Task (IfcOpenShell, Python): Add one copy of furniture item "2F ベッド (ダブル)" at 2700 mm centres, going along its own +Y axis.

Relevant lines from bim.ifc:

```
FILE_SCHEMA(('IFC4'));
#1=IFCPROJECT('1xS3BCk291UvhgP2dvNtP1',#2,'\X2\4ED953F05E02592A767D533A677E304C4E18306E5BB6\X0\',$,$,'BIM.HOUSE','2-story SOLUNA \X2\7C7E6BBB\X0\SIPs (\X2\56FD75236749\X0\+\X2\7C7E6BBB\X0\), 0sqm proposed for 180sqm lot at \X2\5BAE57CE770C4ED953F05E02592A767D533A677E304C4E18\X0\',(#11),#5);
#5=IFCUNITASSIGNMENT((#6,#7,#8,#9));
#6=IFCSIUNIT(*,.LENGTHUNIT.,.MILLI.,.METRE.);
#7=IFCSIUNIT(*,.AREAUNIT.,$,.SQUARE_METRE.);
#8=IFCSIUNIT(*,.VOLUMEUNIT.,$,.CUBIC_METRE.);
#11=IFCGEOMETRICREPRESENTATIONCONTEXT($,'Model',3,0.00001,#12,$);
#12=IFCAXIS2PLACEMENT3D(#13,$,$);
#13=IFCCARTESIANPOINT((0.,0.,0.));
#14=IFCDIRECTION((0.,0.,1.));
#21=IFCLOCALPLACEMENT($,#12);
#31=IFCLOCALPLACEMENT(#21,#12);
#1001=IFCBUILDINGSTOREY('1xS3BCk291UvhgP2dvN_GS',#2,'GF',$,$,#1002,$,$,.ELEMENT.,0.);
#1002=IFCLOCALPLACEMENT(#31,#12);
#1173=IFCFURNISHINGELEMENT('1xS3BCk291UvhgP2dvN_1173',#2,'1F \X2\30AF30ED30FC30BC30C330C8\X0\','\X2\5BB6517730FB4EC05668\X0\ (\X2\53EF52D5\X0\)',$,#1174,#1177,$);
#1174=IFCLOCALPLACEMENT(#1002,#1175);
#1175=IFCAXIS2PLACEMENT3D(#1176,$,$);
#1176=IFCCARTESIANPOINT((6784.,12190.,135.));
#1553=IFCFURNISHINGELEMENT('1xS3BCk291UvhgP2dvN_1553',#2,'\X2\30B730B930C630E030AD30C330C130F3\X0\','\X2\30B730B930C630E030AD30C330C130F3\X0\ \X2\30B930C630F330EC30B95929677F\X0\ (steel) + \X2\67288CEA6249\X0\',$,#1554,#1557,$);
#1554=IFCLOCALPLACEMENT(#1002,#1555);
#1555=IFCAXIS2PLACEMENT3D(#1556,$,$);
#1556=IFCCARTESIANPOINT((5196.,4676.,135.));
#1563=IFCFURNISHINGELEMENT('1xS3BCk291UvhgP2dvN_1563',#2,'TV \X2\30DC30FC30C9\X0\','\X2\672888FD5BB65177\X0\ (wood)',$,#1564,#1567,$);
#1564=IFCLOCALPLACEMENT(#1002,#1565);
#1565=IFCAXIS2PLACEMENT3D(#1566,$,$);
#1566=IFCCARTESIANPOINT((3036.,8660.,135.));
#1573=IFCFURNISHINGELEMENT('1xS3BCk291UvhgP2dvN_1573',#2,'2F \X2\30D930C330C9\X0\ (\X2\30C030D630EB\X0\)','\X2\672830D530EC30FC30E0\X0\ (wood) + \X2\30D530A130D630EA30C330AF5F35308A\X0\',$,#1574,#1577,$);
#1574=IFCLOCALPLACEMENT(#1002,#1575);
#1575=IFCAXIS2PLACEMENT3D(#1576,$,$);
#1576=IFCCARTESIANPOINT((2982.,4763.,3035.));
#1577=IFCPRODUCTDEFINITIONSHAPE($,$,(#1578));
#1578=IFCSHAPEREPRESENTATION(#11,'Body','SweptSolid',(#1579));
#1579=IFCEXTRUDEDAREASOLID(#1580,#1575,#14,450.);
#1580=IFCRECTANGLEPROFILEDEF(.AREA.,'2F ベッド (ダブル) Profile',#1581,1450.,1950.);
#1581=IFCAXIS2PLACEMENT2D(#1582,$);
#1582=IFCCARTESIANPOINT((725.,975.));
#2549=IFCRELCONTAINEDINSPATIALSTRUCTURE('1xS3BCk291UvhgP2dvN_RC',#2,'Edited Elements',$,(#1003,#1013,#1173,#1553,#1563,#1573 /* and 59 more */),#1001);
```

```python
import ifcopenshell
import ifcopenshell.api.geometry
import ifcopenshell.api.root
import ifcopenshell.util.element
import ifcopenshell.util.placement
import ifcopenshell.util.unit

model = ifcopenshell.open("bim.ifc")
unit_scale = ifcopenshell.util.unit.calculate_unit_scale(model)


def reuse_history(source, copy):
    """copy_class also copies each property set's owner history, people and application; keep the originals."""
    for rel in copy.IsDefinedBy:
        if rel.is_a("IfcRelDefinesByProperties") and (history := rel.RelatingPropertyDefinition.OwnerHistory):
            rel.RelatingPropertyDefinition.OwnerHistory = source.OwnerHistory
            ifcopenshell.util.element.remove_deep2(model, history)


source = model.by_guid("1xS3BCk291UvhgP2dvN_1573")
base = ifcopenshell.util.placement.get_local_placement(source.ObjectPlacement)
step = base[:3, 1] * 2.7 / unit_scale

for i in range(1, 2):
    copy = ifcopenshell.api.root.copy_class(model, product=source)
    copy.Representation = ifcopenshell.util.element.copy_deep(
        model, source.Representation, exclude=["IfcGeometricRepresentationContext", "IfcRepresentationMap"]
    )
    reuse_history(source, copy)
    matrix = base.copy()
    matrix[:3, 3] += i * step
    print("added at", matrix[:3, 3].round(3) + 0.0)
    ifcopenshell.api.geometry.edit_object_placement(model, product=copy, matrix=matrix, is_si=False)

model.write("bim-out.ifc")
```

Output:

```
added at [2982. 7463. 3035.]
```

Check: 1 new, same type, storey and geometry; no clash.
